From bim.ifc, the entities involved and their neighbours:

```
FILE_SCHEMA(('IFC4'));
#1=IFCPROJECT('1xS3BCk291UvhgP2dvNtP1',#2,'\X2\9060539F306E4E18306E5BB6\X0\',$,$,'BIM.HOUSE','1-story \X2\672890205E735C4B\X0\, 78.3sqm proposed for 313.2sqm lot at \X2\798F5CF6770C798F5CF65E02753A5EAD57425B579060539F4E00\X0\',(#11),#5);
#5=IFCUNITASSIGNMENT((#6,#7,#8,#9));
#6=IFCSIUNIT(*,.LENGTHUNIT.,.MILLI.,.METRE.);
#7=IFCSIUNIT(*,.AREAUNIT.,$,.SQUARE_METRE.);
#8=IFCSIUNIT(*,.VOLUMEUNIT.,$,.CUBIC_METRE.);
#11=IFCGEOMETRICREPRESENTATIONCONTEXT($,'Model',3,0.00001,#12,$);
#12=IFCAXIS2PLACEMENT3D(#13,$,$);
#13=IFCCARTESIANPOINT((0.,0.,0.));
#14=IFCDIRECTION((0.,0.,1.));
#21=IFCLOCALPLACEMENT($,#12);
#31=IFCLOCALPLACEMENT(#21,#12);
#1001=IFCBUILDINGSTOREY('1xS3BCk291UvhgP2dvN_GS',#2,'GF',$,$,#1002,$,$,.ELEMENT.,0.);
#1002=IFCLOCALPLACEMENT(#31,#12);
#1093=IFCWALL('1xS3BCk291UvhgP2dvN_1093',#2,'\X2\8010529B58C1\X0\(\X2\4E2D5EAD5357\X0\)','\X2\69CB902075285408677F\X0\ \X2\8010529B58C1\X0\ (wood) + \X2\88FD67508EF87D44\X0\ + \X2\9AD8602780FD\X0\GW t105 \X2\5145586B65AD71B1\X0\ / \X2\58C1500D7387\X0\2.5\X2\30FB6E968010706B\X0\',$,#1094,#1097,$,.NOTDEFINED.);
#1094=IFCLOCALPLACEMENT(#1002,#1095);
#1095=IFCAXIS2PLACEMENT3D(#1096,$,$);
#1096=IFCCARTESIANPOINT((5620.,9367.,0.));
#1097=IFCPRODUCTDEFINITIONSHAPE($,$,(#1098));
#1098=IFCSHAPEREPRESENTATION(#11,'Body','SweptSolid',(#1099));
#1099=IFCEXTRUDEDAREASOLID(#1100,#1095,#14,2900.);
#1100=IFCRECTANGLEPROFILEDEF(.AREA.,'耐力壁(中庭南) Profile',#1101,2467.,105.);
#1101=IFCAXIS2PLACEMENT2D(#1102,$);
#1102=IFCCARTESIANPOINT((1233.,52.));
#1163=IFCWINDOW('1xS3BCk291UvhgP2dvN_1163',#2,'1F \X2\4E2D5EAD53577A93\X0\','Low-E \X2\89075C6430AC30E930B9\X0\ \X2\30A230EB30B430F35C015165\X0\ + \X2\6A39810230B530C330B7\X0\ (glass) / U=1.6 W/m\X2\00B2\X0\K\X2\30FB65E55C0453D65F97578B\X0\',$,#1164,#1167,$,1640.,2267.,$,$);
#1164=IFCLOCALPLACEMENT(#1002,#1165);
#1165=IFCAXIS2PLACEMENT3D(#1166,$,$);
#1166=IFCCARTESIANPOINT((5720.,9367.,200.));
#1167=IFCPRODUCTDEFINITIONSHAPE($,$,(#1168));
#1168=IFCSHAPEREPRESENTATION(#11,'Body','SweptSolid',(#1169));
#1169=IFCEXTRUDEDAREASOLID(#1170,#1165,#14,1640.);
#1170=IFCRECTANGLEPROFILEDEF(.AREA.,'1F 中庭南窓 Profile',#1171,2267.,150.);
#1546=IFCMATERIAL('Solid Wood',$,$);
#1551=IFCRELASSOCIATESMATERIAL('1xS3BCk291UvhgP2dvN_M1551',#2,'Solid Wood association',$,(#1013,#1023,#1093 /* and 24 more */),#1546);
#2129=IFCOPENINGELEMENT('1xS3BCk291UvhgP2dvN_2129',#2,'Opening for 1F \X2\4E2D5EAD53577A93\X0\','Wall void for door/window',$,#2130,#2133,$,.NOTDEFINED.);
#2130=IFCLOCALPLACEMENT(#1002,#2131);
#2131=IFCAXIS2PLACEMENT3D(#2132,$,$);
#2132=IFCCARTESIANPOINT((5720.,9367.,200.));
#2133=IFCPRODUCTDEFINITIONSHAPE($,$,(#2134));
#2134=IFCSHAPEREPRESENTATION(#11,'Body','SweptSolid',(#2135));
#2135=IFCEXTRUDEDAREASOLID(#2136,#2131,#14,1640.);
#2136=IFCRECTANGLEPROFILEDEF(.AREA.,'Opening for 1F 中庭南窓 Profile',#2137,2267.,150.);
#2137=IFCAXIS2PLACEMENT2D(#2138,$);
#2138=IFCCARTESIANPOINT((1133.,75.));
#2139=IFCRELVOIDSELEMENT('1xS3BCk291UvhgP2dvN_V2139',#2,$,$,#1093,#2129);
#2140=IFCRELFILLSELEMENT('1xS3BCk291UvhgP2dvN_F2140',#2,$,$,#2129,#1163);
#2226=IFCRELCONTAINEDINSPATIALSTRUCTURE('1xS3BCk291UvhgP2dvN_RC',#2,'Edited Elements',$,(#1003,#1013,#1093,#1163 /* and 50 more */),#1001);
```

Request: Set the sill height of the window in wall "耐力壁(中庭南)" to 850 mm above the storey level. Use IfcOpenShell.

```python
import numpy as np
import ifcopenshell
import ifcopenshell.api.geometry
import ifcopenshell.geom
import ifcopenshell.util.element
import ifcopenshell.util.placement
import ifcopenshell.util.shape
import ifcopenshell.util.unit

model = ifcopenshell.open("bim.ifc")
unit_scale = ifcopenshell.util.unit.calculate_unit_scale(model)

window = model.by_id(1163)
opening = window.FillsVoids[0].RelatingOpeningElement
storey = ifcopenshell.util.element.get_container(window, ifc_class="IfcBuildingStorey")
level = ifcopenshell.util.placement.get_local_placement(storey.ObjectPlacement)[2, 3]

# The opening's origin need not be at the sill, so measure its lowest point.
shape = ifcopenshell.geom.create_shape(ifcopenshell.geom.settings(), opening)
bottom = ifcopenshell.util.shape.get_shape_bottom_elevation(shape, shape.geometry) / unit_scale
dz = level + 0.85 / unit_scale - bottom

shift = np.array([0.0, 0.0, dz])
# The window is not placed relative to its opening, so move both.
for product in (opening, window):
    matrix = ifcopenshell.util.placement.get_local_placement(product.ObjectPlacement)
    matrix[:3, 3] += shift
    ifcopenshell.api.geometry.edit_object_placement(model, product=product, matrix=matrix, is_si=False)

print(f"moved by {dz * unit_scale:+.3f} m")

model.write("bim-out.ifc")
```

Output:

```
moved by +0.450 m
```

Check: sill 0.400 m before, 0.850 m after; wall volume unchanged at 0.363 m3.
